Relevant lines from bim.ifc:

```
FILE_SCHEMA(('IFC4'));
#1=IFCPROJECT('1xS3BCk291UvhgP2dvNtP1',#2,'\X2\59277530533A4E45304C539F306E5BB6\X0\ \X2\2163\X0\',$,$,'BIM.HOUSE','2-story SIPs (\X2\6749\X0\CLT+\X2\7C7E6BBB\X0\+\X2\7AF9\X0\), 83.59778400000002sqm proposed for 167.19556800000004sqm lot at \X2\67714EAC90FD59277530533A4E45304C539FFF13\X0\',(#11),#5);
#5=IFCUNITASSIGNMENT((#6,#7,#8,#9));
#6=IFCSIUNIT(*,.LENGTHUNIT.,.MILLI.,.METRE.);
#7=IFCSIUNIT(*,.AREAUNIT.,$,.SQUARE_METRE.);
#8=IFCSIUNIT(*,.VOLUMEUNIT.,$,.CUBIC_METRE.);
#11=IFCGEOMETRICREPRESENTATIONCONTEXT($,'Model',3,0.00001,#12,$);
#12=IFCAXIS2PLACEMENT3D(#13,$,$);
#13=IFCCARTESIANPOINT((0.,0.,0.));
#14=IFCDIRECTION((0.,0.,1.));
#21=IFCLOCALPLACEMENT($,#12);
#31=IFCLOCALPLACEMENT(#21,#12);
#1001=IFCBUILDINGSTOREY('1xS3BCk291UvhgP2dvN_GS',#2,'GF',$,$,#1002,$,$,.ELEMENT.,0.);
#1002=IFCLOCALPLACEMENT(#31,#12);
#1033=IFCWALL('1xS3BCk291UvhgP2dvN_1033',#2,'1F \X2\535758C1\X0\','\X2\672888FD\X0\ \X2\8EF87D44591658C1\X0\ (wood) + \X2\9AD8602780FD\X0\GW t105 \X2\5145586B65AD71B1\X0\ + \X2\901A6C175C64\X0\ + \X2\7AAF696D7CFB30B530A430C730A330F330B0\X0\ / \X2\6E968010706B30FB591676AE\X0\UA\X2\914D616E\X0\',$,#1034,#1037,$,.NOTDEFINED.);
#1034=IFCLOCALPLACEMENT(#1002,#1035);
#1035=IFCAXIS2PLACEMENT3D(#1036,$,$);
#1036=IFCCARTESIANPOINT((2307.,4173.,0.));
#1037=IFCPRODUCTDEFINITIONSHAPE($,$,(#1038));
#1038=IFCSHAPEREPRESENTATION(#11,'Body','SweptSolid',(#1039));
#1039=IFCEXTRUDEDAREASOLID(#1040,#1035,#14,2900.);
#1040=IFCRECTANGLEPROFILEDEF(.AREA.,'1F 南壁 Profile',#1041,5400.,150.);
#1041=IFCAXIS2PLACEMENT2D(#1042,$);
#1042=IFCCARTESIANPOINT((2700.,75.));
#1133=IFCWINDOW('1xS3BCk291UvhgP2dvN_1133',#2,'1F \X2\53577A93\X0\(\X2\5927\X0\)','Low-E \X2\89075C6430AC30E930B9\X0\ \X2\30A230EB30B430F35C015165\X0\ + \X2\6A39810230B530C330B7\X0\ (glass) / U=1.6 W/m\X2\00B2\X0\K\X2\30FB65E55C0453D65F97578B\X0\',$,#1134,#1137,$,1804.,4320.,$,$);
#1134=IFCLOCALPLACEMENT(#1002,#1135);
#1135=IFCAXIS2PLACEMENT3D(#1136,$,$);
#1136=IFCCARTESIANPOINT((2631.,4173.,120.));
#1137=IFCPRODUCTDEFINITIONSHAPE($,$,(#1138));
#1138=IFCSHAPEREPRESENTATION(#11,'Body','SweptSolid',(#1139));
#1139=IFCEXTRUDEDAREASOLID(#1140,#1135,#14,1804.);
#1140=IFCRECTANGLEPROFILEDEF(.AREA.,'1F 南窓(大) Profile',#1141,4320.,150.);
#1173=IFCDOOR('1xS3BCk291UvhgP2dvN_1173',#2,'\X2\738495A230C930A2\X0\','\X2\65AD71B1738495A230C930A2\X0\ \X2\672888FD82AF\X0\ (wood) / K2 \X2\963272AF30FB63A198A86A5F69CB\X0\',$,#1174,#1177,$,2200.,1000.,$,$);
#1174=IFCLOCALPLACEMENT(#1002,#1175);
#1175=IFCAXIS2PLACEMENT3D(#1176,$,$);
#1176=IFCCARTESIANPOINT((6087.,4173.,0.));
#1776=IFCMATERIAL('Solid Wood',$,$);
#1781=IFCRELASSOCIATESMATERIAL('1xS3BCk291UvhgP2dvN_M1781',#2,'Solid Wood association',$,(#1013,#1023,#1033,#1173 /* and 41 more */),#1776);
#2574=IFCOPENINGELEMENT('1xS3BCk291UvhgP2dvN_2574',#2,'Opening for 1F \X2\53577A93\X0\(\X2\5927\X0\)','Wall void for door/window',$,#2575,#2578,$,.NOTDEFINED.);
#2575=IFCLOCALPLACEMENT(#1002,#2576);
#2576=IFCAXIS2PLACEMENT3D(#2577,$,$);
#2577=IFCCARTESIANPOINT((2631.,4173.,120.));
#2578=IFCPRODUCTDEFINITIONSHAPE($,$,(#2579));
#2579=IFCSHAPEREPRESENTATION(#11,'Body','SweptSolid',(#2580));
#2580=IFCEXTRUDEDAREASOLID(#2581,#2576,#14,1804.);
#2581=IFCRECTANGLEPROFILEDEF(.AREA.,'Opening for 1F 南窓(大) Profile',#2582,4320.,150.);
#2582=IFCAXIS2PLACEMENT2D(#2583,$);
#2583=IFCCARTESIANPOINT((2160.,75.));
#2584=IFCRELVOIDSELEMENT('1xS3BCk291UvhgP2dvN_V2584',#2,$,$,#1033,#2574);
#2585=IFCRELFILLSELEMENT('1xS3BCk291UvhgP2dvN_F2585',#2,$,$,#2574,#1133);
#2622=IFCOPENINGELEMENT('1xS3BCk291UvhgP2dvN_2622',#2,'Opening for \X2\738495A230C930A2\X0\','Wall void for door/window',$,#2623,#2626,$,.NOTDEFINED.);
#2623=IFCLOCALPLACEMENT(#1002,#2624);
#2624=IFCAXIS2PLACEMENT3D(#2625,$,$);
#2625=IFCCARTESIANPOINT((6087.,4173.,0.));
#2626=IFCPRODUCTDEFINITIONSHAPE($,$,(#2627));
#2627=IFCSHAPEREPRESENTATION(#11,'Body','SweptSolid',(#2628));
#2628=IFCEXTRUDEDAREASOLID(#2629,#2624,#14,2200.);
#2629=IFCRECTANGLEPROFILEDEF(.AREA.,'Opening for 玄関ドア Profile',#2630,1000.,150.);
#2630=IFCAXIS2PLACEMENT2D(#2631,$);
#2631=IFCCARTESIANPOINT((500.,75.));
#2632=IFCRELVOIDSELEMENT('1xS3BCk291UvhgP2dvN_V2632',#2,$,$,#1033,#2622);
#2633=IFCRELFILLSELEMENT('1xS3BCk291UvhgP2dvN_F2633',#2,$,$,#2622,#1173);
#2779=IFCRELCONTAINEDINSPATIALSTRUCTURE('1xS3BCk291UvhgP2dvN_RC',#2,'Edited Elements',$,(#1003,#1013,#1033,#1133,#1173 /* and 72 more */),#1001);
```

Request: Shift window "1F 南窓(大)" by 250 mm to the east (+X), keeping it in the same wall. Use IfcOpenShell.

```python
import ifcopenshell
import ifcopenshell.api.geometry
import ifcopenshell.util.placement
import ifcopenshell.util.unit

model = ifcopenshell.open("bim.ifc")
unit_scale = ifcopenshell.util.unit.calculate_unit_scale(model)

window = model.by_guid("1xS3BCk291UvhgP2dvN_1133")
opening = window.FillsVoids[0].RelatingOpeningElement
wall = opening.VoidsElements[0].RelatingBuildingElement

wall_matrix = ifcopenshell.util.placement.get_local_placement(wall.ObjectPlacement)
shift = wall_matrix[:3, 0] * 0.25 / unit_scale
before = ifcopenshell.util.placement.get_local_placement(window.ObjectPlacement)[:3, 3].copy()

# The window is not placed relative to its opening, so move both.
for product in (opening, window):
    matrix = ifcopenshell.util.placement.get_local_placement(product.ObjectPlacement)
    matrix[:3, 3] += shift
    ifcopenshell.api.geometry.edit_object_placement(model, product=product, matrix=matrix, is_si=False)

after = ifcopenshell.util.placement.get_local_placement(window.ObjectPlacement)[:3, 3]
print("window moved by", (after - before).round(3) + 0.0)

model.write("bim_updated.ifc")
```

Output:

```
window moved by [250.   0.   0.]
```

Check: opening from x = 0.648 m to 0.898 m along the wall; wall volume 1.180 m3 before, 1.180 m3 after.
